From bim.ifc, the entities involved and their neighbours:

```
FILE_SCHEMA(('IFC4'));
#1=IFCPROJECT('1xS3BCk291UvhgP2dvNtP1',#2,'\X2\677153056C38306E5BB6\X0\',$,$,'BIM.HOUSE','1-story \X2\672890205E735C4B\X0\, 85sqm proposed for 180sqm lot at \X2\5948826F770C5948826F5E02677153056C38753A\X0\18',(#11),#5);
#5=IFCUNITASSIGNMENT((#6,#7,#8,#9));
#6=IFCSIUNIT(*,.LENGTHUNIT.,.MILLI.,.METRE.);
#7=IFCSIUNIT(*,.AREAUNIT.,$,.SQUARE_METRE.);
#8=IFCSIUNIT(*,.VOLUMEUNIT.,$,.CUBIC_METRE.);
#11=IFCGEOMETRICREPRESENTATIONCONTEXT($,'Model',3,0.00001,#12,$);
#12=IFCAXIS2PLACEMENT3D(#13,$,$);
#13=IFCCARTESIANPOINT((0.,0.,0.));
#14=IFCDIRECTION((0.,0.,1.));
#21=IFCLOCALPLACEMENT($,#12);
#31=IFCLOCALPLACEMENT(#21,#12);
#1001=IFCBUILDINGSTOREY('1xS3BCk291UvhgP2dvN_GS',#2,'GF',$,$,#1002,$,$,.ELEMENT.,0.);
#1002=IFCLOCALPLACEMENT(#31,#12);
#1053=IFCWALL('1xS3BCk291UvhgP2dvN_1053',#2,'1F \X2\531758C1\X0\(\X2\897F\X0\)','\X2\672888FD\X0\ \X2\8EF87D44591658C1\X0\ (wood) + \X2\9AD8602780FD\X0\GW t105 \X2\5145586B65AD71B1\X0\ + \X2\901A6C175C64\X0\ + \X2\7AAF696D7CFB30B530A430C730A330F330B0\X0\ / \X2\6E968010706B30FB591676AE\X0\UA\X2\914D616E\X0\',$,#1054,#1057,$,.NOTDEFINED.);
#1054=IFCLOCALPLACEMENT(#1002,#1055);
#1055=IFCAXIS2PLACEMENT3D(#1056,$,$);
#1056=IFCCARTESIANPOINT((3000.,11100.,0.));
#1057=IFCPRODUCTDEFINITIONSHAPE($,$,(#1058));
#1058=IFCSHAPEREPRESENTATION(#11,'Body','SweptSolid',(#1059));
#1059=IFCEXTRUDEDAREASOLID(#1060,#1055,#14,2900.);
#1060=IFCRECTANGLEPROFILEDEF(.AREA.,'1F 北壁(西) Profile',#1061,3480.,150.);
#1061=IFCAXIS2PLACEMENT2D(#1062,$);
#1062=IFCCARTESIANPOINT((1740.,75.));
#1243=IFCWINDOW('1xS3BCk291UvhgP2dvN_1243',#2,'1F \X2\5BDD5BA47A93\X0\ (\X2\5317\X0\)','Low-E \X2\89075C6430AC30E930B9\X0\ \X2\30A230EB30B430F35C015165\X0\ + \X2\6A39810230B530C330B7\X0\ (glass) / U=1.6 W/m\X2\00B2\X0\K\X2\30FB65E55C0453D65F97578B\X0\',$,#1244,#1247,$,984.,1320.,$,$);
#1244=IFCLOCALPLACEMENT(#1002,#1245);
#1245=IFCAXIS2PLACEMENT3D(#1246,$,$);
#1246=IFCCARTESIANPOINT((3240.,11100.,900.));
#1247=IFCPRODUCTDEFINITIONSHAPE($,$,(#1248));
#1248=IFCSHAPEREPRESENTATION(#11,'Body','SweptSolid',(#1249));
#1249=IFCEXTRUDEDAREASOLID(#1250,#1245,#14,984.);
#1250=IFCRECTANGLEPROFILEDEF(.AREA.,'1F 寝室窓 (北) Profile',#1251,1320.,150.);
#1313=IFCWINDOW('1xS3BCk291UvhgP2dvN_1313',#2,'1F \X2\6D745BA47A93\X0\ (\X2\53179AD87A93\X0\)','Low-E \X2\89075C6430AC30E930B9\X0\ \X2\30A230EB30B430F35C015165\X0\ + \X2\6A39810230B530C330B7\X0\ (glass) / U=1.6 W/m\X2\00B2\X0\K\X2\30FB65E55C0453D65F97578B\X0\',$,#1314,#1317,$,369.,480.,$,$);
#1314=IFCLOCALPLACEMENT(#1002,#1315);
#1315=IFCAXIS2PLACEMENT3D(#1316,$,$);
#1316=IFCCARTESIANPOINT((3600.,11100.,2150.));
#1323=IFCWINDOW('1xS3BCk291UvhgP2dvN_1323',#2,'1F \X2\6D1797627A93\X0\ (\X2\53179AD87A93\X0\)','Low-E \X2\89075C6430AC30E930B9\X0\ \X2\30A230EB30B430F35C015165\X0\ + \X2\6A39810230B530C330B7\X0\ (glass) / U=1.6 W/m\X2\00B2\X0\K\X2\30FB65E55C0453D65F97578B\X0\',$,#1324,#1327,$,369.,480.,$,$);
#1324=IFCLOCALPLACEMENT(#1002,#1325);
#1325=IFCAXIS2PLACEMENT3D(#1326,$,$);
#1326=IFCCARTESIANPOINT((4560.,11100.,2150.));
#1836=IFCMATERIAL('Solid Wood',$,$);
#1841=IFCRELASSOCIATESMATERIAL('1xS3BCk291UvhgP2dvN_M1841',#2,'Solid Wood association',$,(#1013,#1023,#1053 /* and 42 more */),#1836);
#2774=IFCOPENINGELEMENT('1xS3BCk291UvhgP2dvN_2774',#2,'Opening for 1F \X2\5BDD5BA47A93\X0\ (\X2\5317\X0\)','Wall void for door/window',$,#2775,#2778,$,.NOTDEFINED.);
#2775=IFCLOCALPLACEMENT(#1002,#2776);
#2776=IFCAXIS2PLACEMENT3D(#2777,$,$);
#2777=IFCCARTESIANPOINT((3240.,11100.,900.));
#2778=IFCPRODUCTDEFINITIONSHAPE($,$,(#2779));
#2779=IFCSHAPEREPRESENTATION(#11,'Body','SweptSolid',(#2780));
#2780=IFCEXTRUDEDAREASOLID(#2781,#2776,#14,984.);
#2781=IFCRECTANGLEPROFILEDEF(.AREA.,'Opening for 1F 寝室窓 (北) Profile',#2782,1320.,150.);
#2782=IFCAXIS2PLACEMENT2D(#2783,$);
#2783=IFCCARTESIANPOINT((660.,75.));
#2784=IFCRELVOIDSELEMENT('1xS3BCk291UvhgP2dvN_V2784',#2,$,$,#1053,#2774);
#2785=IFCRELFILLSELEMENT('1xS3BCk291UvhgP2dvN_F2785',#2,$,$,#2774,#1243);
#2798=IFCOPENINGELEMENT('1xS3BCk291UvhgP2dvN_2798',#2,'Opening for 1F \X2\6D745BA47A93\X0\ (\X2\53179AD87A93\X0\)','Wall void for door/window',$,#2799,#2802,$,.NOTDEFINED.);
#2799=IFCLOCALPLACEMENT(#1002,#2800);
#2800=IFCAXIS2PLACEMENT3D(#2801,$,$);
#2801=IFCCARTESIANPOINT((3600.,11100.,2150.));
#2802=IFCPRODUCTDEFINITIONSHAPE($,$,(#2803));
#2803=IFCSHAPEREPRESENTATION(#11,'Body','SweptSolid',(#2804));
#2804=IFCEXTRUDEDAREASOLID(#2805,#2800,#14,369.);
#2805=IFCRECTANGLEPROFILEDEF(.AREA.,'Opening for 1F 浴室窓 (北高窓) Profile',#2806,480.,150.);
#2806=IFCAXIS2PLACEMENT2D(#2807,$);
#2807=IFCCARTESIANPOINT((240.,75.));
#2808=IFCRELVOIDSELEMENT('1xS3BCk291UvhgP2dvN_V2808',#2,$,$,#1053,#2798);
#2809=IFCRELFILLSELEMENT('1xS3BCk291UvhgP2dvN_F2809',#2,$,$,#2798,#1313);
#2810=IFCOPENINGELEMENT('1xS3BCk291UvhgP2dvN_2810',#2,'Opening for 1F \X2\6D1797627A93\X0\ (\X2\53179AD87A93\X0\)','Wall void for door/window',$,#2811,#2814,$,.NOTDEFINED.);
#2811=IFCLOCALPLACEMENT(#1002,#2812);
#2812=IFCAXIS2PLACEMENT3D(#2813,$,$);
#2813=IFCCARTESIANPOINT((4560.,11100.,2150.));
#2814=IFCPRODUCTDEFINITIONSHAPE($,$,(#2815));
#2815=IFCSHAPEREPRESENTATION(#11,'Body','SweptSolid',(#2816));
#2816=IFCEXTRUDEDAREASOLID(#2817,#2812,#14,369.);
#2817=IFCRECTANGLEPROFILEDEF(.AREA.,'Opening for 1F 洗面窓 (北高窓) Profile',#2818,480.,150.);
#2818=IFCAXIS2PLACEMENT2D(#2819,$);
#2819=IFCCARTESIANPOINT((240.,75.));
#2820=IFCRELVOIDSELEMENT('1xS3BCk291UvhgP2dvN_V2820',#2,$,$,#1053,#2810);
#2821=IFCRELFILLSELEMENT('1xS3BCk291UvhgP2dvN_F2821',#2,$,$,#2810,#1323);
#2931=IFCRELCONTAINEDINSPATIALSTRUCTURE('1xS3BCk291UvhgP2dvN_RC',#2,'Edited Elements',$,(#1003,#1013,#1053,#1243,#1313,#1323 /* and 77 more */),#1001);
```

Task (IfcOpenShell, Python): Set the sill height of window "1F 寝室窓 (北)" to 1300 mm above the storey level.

```python
import numpy as np
import ifcopenshell
import ifcopenshell.api.geometry
import ifcopenshell.geom
import ifcopenshell.util.element
import ifcopenshell.util.placement
import ifcopenshell.util.shape
import ifcopenshell.util.unit

model = ifcopenshell.open("bim.ifc")
unit_scale = ifcopenshell.util.unit.calculate_unit_scale(model)

window = model.by_guid("1xS3BCk291UvhgP2dvN_1243")
opening = window.FillsVoids[0].RelatingOpeningElement
storey = ifcopenshell.util.element.get_container(window, ifc_class="IfcBuildingStorey")
level = ifcopenshell.util.placement.get_local_placement(storey.ObjectPlacement)[2, 3]

# The opening's origin need not be at the sill, so measure its lowest point.
shape = ifcopenshell.geom.create_shape(ifcopenshell.geom.settings(), opening)
bottom = ifcopenshell.util.shape.get_shape_bottom_elevation(shape, shape.geometry) / unit_scale
dz = level + 1.3 / unit_scale - bottom

shift = np.array([0.0, 0.0, dz])
# The window is not placed relative to its opening, so move both.
for product in (opening, window):
    matrix = ifcopenshell.util.placement.get_local_placement(product.ObjectPlacement)
    matrix[:3, 3] += shift
    ifcopenshell.api.geometry.edit_object_placement(model, product=product, matrix=matrix, is_si=False)

print(f"moved by {dz * unit_scale:+.3f} m")

model.write("bim_v2.ifc")
```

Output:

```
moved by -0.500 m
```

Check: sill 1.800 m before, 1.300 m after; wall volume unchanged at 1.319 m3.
